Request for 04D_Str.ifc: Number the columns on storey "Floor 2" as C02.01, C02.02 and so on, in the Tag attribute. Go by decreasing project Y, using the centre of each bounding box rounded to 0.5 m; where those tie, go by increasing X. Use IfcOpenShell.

First a look at what the model holds.

```python
import ifcopenshell
import ifcopenshell.util.element
import ifcopenshell.util.placement

model = ifcopenshell.open("04D_Str.ifc")
print(model.schema)
storey = next(s for s in model.by_type("IfcBuildingStorey") if s.Name == "Floor 2")
columns = [e for e in ifcopenshell.util.element.get_decomposition(storey) if e.is_a("IfcColumn")]
for e in sorted(columns, key=lambda e: e.id()):
    origin = ifcopenshell.util.placement.get_local_placement(e.ObjectPlacement)[:3, 3]
    print(e.id(), e.Tag, e.Name, origin.round(2) + 0.0, sep=" | ")
```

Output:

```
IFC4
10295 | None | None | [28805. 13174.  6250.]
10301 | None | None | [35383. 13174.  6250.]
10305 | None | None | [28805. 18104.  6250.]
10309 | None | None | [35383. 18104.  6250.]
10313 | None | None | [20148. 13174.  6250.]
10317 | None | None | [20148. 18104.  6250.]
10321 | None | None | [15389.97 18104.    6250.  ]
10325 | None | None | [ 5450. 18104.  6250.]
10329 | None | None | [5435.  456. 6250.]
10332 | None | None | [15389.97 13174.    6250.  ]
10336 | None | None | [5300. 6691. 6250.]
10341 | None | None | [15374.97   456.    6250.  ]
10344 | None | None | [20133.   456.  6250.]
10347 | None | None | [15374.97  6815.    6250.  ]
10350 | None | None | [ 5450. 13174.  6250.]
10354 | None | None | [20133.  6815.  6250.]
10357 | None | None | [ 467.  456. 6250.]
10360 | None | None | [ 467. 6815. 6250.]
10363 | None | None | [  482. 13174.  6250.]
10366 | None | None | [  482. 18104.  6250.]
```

```python
import ifcopenshell
import ifcopenshell.geom
import ifcopenshell.util.element
import ifcopenshell.util.shape

model = ifcopenshell.open("04D_Str.ifc")
settings = ifcopenshell.geom.settings()
settings.set("use-world-coords", True)


def centre(element):
    shape = ifcopenshell.geom.create_shape(settings, element)
    return ifcopenshell.util.shape.get_bbox_centroid(shape.geometry)


storey = next(s for s in model.by_type("IfcBuildingStorey") if s.Name == "Floor 2")
columns = [e for e in ifcopenshell.util.element.get_decomposition(storey) if e.is_a("IfcColumn")]

# Insertion points can sit at a corner or the storey origin, so sort by the geometry (in metres).
centres = {e: centre(e) for e in columns}
columns.sort(key=lambda e: (-round(centres[e][1] / 0.5), centres[e][0]))

for i, e in enumerate(columns, start=1):
    number = f"C02.{i:02d}"
    e.Tag = number
    print(e.id(), number)

model.write("04D_Str-out.ifc")
```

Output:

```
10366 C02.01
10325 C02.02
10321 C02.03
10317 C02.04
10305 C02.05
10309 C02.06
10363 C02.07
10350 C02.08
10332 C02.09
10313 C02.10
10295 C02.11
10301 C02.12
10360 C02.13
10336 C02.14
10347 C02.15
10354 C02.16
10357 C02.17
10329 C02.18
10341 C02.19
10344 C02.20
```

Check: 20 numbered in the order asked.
